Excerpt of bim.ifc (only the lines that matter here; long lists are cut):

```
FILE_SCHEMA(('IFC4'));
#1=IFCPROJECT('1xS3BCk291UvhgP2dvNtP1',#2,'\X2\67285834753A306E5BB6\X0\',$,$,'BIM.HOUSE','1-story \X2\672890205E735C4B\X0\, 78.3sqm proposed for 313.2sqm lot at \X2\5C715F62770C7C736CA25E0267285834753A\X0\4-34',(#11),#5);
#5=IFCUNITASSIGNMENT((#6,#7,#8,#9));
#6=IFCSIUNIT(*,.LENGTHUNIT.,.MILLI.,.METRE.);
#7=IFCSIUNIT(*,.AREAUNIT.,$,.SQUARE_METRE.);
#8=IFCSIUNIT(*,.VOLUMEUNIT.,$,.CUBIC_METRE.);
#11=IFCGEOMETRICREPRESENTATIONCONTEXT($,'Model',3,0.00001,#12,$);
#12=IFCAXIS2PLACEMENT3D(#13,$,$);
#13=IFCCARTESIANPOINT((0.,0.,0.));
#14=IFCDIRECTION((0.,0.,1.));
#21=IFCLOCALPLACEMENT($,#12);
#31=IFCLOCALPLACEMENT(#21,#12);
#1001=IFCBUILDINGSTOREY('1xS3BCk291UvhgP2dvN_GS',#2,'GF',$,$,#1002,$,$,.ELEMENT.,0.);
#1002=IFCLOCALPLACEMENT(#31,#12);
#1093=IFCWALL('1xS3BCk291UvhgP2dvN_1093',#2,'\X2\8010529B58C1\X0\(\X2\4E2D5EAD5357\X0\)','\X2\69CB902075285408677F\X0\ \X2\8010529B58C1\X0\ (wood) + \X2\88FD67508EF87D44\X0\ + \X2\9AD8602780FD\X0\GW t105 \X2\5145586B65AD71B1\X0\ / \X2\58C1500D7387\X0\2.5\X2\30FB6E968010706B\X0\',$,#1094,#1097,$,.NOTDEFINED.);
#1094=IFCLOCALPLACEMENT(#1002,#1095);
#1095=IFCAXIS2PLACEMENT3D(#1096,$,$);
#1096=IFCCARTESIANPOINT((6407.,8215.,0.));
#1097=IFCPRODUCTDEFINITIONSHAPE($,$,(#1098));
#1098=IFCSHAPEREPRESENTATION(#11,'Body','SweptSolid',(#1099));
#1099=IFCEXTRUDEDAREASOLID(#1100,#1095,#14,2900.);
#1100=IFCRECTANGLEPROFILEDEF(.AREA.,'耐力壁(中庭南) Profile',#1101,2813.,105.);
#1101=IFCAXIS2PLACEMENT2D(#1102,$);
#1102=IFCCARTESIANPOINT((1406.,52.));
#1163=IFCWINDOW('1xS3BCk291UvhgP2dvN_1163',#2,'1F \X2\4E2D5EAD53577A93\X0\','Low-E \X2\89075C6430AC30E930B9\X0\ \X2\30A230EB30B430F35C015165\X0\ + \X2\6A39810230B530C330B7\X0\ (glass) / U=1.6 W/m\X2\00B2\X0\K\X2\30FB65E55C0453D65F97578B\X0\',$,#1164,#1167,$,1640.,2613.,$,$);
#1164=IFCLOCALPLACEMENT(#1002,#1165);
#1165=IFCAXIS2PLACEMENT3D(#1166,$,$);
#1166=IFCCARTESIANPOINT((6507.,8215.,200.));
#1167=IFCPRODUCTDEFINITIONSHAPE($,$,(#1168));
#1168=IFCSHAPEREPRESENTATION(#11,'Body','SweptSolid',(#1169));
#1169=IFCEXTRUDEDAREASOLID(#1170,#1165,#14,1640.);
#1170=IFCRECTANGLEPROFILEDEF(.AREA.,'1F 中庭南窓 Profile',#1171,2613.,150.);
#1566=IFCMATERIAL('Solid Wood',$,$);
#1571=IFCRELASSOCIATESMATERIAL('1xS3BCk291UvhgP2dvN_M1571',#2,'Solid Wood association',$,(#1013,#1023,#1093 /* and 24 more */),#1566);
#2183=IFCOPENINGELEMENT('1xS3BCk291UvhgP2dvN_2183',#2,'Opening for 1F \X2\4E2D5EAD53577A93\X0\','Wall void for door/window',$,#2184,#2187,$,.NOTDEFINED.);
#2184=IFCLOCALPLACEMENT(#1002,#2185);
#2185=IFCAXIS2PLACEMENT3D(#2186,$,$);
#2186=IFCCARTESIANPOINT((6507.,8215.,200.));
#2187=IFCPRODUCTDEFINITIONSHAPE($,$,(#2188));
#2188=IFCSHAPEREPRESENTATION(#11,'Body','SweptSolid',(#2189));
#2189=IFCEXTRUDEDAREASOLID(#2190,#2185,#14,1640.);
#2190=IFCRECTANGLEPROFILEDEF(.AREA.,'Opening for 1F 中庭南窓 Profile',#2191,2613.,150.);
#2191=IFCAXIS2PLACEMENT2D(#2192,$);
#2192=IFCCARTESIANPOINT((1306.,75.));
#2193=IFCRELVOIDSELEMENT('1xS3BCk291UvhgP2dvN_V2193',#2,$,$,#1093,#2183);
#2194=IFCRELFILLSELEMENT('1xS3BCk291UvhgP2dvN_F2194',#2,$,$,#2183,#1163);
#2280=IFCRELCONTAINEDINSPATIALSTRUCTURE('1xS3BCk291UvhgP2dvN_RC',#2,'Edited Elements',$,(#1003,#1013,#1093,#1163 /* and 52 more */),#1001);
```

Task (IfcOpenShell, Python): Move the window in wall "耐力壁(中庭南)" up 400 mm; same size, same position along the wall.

```python
import numpy as np
import ifcopenshell
import ifcopenshell.api.geometry
import ifcopenshell.util.placement
import ifcopenshell.util.unit

model = ifcopenshell.open("bim.ifc")
unit_scale = ifcopenshell.util.unit.calculate_unit_scale(model)

window = model.by_guid("1xS3BCk291UvhgP2dvN_1163")
opening = window.FillsVoids[0].RelatingOpeningElement
dz = 400.0

shift = np.array([0.0, 0.0, dz])
# The window is not placed relative to its opening, so move both.
for product in (opening, window):
    matrix = ifcopenshell.util.placement.get_local_placement(product.ObjectPlacement)
    matrix[:3, 3] += shift
    ifcopenshell.api.geometry.edit_object_placement(model, product=product, matrix=matrix, is_si=False)

print(f"moved by {dz * unit_scale:+.3f} m")

model.write("bim_updated.ifc")
```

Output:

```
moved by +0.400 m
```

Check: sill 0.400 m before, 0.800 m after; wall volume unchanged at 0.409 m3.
